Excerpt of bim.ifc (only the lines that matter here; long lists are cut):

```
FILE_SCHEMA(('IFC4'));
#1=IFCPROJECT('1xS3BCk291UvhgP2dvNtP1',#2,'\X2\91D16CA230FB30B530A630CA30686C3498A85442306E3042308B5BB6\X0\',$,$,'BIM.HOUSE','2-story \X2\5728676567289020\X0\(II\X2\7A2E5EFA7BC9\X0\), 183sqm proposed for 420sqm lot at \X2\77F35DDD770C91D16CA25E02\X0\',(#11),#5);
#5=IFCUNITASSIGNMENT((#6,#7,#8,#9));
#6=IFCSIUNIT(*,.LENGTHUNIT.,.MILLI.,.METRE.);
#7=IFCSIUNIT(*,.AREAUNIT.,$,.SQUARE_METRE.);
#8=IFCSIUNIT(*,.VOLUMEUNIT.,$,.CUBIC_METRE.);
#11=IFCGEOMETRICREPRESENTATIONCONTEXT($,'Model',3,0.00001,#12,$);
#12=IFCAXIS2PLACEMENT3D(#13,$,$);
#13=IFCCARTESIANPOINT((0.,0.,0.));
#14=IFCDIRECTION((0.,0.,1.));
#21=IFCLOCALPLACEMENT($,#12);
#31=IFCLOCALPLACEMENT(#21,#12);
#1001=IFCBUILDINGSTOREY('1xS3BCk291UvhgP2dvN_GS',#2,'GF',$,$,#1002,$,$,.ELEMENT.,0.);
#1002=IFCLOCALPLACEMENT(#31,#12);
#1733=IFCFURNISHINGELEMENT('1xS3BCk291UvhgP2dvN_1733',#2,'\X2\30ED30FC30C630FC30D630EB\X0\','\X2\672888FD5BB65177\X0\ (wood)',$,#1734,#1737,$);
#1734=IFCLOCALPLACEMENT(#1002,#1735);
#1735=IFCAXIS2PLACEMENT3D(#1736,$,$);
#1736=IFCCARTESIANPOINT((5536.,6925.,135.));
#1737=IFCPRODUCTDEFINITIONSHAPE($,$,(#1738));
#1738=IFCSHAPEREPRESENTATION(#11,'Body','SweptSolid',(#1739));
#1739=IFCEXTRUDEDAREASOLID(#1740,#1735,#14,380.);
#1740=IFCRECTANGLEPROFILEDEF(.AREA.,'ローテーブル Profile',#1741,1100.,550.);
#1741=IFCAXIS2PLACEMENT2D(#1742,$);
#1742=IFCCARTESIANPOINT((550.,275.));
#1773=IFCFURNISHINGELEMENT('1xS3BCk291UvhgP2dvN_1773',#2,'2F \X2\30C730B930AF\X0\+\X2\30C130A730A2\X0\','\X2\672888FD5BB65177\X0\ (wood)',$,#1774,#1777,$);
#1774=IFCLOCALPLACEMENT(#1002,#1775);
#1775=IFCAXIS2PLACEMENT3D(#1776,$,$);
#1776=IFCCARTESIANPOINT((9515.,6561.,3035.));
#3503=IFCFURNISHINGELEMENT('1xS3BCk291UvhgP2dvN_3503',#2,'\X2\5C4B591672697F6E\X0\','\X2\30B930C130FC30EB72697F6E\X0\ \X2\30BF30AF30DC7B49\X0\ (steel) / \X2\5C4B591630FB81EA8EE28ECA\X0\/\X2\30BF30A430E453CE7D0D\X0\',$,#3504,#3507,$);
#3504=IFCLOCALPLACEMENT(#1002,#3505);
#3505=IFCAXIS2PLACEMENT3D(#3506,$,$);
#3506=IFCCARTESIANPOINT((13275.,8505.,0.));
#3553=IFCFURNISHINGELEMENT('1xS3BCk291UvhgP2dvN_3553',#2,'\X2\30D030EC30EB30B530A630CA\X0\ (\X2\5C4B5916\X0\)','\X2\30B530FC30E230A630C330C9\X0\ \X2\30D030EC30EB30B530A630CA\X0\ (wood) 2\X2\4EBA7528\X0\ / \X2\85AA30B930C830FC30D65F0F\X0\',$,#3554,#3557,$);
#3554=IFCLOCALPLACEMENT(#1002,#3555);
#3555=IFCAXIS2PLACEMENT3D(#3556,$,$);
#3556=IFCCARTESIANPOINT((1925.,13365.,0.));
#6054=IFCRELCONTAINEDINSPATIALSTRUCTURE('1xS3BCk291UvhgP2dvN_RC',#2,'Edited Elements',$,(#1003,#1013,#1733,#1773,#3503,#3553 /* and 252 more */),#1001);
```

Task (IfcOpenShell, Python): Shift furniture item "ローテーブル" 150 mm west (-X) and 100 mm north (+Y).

```python
import ifcopenshell
import ifcopenshell.api.geometry
import ifcopenshell.util.placement

model = ifcopenshell.open("bim.ifc")

item = model.by_guid("1xS3BCk291UvhgP2dvN_1733")
matrix = ifcopenshell.util.placement.get_local_placement(item.ObjectPlacement)
matrix[0, 3] -= 150.0
matrix[1, 3] += 100.0
ifcopenshell.api.geometry.edit_object_placement(model, product=item, matrix=matrix, is_si=False)

print(ifcopenshell.util.placement.get_local_placement(item.ObjectPlacement).round(3) + 0.0)

model.write("bim_v2.ifc")
```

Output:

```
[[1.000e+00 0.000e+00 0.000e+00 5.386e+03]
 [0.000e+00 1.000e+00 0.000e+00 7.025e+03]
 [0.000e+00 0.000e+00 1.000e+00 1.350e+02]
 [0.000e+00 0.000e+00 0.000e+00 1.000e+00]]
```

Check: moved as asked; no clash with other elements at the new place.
